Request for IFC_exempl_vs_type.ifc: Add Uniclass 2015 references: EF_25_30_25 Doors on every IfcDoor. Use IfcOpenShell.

First a look at what the model holds.

```python
import ifcopenshell

model = ifcopenshell.open("IFC_exempl_vs_type.ifc")
print(model.schema)
print("classifications:", [c.Name for c in model.by_type("IfcClassification")])
for ifc_class in ("IfcDoor", "IfcRoof", "IfcStair", "IfcWall", "IfcWindow"):
    print(ifc_class, len(model.by_type(ifc_class)))
```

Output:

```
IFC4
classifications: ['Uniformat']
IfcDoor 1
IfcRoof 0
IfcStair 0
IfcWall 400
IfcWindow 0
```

```python
import ifcopenshell
import ifcopenshell.api.classification

model = ifcopenshell.open("IFC_exempl_vs_type.ifc")

system = ifcopenshell.api.classification.add_classification(model, classification="Uniclass 2015")

codes = {
    "IfcDoor": ("EF_25_30_25", "Doors"),
}
for ifc_class, (code, name) in codes.items():
    products = model.by_type(ifc_class)
    ifcopenshell.api.classification.add_reference(
        model, products=products, classification=system, identification=code, name=name
    )
    print(code, len(products))

model.write("IFC_exempl_vs_type_v2.ifc")
```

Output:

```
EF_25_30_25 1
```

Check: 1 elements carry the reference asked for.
